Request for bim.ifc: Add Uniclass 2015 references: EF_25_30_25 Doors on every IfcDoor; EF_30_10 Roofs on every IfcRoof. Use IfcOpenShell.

First a look at what the model holds.

```python
import ifcopenshell

model = ifcopenshell.open("bim.ifc")
print(model.schema)
print("classifications:", [c.Name for c in model.by_type("IfcClassification")])
for ifc_class in ("IfcDoor", "IfcRoof", "IfcStair", "IfcWall", "IfcWindow"):
    print(ifc_class, len(model.by_type(ifc_class)))
```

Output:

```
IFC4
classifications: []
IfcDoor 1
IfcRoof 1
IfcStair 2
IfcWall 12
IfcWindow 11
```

```python
import ifcopenshell
import ifcopenshell.api.classification

model = ifcopenshell.open("bim.ifc")

system = ifcopenshell.api.classification.add_classification(model, classification="Uniclass 2015")

codes = {
    "IfcDoor": ("EF_25_30_25", "Doors"),
    "IfcRoof": ("EF_30_10", "Roofs"),
}
for ifc_class, (code, name) in codes.items():
    products = model.by_type(ifc_class)
    ifcopenshell.api.classification.add_reference(
        model, products=products, classification=system, identification=code, name=name
    )
    print(code, len(products))

model.write("bim-out.ifc")
```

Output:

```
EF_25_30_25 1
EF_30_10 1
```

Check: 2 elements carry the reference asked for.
